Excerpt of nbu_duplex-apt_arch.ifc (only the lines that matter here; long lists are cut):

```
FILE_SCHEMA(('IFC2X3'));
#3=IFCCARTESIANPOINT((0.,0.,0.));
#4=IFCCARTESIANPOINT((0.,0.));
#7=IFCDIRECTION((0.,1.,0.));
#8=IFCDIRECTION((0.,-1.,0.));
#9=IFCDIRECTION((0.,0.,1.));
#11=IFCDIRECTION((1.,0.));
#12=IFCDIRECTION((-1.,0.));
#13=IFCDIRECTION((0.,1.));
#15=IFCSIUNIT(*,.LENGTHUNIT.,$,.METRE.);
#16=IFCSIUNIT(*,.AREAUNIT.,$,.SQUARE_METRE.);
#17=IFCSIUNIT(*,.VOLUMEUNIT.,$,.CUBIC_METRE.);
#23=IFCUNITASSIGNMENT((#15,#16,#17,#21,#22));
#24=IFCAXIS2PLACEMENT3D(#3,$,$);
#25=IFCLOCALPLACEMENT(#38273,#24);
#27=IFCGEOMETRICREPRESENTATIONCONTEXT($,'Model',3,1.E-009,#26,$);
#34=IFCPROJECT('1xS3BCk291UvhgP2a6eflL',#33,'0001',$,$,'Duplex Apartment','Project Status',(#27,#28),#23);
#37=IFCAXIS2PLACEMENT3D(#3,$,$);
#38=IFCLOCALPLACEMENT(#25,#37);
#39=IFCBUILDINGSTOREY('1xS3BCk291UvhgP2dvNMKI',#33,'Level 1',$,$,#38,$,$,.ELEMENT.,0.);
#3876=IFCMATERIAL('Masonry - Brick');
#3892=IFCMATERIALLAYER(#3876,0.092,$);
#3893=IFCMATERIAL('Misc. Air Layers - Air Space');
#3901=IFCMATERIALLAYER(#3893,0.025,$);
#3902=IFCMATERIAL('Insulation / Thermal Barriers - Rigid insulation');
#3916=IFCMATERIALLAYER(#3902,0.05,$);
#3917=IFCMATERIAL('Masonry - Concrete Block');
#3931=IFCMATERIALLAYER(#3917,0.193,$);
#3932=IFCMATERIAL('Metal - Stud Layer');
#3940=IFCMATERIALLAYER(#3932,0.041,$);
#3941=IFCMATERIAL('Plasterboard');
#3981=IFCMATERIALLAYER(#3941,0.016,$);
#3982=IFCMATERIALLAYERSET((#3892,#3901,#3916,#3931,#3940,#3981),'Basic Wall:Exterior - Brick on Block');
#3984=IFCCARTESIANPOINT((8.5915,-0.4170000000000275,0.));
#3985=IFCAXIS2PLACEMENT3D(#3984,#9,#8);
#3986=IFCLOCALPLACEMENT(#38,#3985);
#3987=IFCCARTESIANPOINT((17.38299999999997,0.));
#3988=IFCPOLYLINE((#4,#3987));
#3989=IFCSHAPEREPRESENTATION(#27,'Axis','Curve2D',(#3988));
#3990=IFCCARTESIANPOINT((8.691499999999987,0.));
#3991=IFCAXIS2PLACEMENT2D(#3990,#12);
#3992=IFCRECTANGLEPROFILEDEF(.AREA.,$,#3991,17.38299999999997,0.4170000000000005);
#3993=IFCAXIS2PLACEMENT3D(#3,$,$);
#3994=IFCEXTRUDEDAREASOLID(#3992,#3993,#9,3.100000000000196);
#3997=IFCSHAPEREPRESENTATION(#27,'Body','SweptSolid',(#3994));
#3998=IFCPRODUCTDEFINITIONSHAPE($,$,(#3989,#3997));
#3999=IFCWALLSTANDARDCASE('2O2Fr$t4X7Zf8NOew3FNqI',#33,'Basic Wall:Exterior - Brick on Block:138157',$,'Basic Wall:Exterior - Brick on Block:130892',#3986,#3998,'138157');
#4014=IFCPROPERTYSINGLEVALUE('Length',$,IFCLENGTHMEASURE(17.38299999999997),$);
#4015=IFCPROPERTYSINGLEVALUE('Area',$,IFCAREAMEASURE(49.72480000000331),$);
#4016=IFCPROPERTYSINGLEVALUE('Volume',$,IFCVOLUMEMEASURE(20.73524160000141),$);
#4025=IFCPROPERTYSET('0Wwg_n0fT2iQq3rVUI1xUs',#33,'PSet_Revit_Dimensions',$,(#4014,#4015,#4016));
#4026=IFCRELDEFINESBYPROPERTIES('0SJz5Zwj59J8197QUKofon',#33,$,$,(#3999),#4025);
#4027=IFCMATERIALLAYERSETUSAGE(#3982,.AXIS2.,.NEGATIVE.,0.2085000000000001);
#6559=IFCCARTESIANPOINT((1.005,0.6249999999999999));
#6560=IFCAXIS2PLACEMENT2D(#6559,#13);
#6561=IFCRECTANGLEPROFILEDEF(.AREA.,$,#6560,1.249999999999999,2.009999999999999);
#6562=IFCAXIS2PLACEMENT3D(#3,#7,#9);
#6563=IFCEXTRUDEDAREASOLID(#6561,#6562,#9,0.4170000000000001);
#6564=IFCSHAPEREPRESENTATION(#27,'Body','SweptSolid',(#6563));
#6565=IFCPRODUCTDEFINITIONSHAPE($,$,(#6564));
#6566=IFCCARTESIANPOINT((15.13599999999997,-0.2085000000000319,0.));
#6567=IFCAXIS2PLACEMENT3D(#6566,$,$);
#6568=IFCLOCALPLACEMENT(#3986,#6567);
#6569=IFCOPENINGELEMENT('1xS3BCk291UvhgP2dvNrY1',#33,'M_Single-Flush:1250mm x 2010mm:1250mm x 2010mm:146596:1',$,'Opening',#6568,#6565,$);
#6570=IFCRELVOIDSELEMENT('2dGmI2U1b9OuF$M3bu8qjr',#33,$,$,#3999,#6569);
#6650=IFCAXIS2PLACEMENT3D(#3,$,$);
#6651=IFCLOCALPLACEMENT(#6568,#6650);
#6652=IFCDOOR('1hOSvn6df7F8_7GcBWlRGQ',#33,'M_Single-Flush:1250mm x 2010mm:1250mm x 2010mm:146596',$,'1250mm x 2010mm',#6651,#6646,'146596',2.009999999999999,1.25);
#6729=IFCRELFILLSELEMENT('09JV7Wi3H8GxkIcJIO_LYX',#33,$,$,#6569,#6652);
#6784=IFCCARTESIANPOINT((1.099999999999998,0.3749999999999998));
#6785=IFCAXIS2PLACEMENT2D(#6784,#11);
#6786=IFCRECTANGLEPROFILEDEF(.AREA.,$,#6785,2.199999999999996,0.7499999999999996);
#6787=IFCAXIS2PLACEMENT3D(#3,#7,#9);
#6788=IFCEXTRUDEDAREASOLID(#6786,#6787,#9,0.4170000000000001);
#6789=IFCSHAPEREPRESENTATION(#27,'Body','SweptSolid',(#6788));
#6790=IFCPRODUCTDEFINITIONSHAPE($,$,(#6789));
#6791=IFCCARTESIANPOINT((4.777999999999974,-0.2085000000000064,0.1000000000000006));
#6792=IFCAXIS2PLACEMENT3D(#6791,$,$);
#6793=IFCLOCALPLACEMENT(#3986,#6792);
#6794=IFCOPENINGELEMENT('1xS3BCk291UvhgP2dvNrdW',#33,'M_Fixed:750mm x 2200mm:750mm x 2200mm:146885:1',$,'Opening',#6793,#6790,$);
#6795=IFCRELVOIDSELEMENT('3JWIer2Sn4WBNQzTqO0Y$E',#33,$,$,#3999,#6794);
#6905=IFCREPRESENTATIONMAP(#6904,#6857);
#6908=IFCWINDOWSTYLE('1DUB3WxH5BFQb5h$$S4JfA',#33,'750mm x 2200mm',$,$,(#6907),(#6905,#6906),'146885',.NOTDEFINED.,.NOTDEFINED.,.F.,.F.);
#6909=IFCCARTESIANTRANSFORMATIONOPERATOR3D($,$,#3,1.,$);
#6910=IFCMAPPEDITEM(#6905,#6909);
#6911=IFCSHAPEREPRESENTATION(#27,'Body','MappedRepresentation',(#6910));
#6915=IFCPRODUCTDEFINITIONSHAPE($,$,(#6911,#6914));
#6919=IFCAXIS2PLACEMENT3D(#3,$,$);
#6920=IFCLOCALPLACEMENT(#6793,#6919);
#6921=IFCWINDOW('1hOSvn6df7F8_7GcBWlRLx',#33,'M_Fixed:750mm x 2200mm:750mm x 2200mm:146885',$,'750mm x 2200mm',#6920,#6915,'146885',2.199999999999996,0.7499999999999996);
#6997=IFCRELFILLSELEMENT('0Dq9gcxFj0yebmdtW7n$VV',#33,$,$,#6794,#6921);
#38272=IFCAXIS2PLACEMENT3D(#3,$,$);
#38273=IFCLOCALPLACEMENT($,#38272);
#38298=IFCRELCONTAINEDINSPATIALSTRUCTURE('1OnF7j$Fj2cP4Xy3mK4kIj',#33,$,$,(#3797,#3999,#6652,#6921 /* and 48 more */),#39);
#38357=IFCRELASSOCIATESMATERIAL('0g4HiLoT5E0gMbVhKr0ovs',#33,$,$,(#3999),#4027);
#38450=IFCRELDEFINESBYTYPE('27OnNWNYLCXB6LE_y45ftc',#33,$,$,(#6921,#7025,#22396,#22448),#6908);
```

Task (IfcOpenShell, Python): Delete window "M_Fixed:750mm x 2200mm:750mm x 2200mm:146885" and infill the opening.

```python
import ifcopenshell
import ifcopenshell.api.feature
import ifcopenshell.api.pset
import ifcopenshell.api.root
import ifcopenshell.geom
import ifcopenshell.util.element
import ifcopenshell.util.shape
import ifcopenshell.util.unit

model = ifcopenshell.open("nbu_duplex-apt_arch.ifc")
area_scale = ifcopenshell.util.unit.calculate_unit_scale(model, "AREAUNIT")
volume_scale = ifcopenshell.util.unit.calculate_unit_scale(model, "VOLUMEUNIT")
settings = ifcopenshell.geom.settings()


def volume(element):
    """Net volume in cubic metres, openings subtracted."""
    shape = ifcopenshell.geom.create_shape(settings, element)
    return ifcopenshell.util.shape.get_volume(shape.geometry)


window = model.by_id(6921)
opening = window.FillsVoids[0].RelatingOpeningElement
wall = opening.VoidsElements[0].RelatingBuildingElement
before = volume(wall)

ifcopenshell.api.root.remove_product(model, product=window)
ifcopenshell.api.feature.remove_feature(model, feature=opening)

after = volume(wall)
thickness = 0.417  # wall thickness in metres

# Update the wall's stored quantities.
pset = model.by_id(ifcopenshell.util.element.get_pset(wall, "PSet_Revit_Dimensions", should_inherit=False)["id"])
ifcopenshell.api.pset.edit_pset(model, pset=pset, properties={
    "Area": model.create_entity("IfcAreaMeasure", after / thickness / area_scale),
    "Volume": model.create_entity("IfcVolumeMeasure", after / volume_scale),
})

print(f"wall volume {before:.3f} -> {after:.3f} m3")

model.write("nbu_duplex-apt_arch_updated.ifc")
```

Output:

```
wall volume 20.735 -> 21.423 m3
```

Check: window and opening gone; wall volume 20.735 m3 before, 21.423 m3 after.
